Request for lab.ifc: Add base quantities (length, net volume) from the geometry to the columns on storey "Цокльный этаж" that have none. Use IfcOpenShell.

First a look at what the model holds.

```python
import ifcopenshell
import ifcopenshell.util.element
import ifcopenshell.util.unit

model = ifcopenshell.open("lab.ifc")
print(model.schema)
for unit_type in ("LENGTHUNIT", "AREAUNIT", "VOLUMEUNIT"):
    print(unit_type, ifcopenshell.util.unit.calculate_unit_scale(model, unit_type))
storey = next(s for s in model.by_type("IfcBuildingStorey") if s.Name == "Цокльный этаж")
columns = [e for e in ifcopenshell.util.element.get_decomposition(storey) if e.is_a("IfcColumn")]
for e in sorted(columns, key=lambda e: e.id()):
    print(e.id(), e.is_a(), e.Name, list(ifcopenshell.util.element.get_psets(e, qtos_only=True)), sep=" | ")
```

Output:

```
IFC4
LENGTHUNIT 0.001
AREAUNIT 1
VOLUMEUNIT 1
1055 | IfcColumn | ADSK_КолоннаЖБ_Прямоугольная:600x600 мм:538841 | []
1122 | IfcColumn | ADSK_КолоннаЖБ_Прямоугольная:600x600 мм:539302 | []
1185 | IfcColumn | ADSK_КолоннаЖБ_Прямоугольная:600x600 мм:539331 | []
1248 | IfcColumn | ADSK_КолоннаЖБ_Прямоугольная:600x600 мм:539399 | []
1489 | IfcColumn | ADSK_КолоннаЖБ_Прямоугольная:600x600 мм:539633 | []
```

```python
import ifcopenshell
import ifcopenshell.api.pset
import ifcopenshell.geom
import ifcopenshell.util.element
import ifcopenshell.util.shape
import ifcopenshell.util.unit

model = ifcopenshell.open("lab.ifc")
unit_scale = ifcopenshell.util.unit.calculate_unit_scale(model)
volume_scale = ifcopenshell.util.unit.calculate_unit_scale(model, "VOLUMEUNIT")
settings = ifcopenshell.geom.settings()

storey = next(s for s in model.by_type("IfcBuildingStorey") if s.Name == "Цокльный этаж")
columns = [e for e in ifcopenshell.util.element.get_decomposition(storey) if e.is_a("IfcColumn")]

for e in sorted(columns, key=lambda e: e.id()):
    if ifcopenshell.util.element.get_psets(e, qtos_only=True, should_inherit=False):
        continue
    # Geometry comes back in metres, in the element's own axes.
    shape = ifcopenshell.geom.create_shape(settings, e)
    values = {
        "Length": ifcopenshell.util.shape.get_z(shape.geometry) / unit_scale,
        "NetVolume": ifcopenshell.util.shape.get_volume(shape.geometry) / volume_scale,
    }
    qto = ifcopenshell.api.pset.add_qto(model, product=e, name="Qto_ColumnBaseQuantities")
    ifcopenshell.api.pset.edit_qto(model, qto=qto, properties=values)
    print(e.id(), {k: round(v, 3) for k, v in values.items()})

model.write("lab_updated.ifc")
```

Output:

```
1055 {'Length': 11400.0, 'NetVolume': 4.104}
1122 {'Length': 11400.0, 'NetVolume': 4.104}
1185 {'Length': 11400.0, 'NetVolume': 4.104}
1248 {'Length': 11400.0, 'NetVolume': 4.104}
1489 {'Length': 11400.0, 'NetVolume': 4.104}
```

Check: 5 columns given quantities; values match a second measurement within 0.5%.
